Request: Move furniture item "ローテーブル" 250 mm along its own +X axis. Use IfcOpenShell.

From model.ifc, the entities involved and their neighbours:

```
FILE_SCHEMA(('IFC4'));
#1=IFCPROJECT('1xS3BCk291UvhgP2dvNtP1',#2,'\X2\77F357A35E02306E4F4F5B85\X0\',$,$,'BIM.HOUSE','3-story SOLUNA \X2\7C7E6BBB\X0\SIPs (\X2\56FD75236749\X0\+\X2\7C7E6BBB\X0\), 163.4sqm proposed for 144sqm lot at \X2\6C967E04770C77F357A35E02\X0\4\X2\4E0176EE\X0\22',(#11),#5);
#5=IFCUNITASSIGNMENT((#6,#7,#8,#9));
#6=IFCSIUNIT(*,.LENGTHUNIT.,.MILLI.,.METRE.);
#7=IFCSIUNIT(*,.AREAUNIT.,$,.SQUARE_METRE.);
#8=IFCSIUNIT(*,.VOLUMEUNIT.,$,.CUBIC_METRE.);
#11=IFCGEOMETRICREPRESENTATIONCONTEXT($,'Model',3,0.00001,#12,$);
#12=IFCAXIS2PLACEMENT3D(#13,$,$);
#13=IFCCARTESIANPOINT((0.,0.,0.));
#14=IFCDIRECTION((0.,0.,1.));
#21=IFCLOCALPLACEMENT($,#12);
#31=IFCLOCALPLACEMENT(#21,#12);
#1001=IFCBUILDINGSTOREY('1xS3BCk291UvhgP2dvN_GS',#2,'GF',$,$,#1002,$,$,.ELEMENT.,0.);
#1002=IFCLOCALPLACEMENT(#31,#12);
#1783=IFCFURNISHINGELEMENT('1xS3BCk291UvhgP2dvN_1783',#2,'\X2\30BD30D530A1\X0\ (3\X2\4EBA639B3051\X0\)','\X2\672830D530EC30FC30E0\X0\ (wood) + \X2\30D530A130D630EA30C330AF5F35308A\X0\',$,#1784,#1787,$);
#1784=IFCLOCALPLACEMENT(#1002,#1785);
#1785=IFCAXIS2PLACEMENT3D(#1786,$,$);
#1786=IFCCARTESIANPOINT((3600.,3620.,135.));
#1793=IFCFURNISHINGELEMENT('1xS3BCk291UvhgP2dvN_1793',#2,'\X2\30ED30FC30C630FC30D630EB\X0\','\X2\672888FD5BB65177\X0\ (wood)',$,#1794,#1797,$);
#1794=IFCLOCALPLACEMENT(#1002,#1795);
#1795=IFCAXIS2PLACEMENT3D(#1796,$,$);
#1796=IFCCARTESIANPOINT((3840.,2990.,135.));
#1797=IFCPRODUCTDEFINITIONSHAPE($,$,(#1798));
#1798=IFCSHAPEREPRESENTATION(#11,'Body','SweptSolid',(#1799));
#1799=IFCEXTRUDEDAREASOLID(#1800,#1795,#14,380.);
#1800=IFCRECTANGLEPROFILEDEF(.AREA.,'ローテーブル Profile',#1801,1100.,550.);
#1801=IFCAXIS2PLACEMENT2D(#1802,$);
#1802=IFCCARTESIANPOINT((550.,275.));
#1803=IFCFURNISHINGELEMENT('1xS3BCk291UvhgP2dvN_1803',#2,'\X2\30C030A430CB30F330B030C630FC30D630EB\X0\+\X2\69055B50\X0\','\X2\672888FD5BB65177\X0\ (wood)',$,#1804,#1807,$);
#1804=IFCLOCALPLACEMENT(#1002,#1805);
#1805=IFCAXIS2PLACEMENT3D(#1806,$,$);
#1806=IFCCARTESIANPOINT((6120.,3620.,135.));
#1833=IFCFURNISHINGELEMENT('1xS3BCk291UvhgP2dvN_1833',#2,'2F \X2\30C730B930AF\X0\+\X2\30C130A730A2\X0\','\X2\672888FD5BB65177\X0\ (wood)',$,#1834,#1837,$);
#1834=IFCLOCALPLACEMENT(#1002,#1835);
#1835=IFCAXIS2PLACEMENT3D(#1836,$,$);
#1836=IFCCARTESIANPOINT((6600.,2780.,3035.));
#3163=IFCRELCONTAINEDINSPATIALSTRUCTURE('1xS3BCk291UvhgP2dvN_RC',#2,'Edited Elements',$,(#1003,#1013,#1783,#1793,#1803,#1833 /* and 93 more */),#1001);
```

```python
import ifcopenshell
import ifcopenshell.api.geometry
import ifcopenshell.util.placement
import ifcopenshell.util.unit

model = ifcopenshell.open("model.ifc")
unit_scale = ifcopenshell.util.unit.calculate_unit_scale(model)

item = model.by_id(1793)
matrix = ifcopenshell.util.placement.get_local_placement(item.ObjectPlacement)
matrix[:3, 3] += matrix[:3, 0] * 0.25 / unit_scale
ifcopenshell.api.geometry.edit_object_placement(model, product=item, matrix=matrix, is_si=False)

print(ifcopenshell.util.placement.get_local_placement(item.ObjectPlacement).round(3) + 0.0)

model.write("model_v2.ifc")
```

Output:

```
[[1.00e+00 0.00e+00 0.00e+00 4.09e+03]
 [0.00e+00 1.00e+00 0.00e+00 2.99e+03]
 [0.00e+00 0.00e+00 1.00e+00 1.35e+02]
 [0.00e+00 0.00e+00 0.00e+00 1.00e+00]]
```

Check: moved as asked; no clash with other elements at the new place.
